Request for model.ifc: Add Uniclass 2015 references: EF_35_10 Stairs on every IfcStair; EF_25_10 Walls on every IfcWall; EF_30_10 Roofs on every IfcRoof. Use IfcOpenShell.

First a look at what the model holds.

```python
import ifcopenshell

model = ifcopenshell.open("model.ifc")
print(model.schema)
print("classifications:", [c.Name for c in model.by_type("IfcClassification")])
for ifc_class in ("IfcDoor", "IfcRoof", "IfcStair", "IfcWall", "IfcWindow"):
    print(ifc_class, len(model.by_type(ifc_class)))
```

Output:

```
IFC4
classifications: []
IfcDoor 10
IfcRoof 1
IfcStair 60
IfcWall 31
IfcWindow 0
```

```python
import ifcopenshell
import ifcopenshell.api.classification

model = ifcopenshell.open("model.ifc")

system = ifcopenshell.api.classification.add_classification(model, classification="Uniclass 2015")

codes = {
    "IfcStair": ("EF_35_10", "Stairs"),
    "IfcWall": ("EF_25_10", "Walls"),
    "IfcRoof": ("EF_30_10", "Roofs"),
}
for ifc_class, (code, name) in codes.items():
    products = model.by_type(ifc_class)
    ifcopenshell.api.classification.add_reference(
        model, products=products, classification=system, identification=code, name=name
    )
    print(code, len(products))

model.write("model-out.ifc")
```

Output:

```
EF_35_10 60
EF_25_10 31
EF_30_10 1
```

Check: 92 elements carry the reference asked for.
